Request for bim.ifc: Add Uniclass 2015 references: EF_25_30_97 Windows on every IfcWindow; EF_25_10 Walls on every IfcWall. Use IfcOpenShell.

First a look at what the model holds.

```python
import ifcopenshell

model = ifcopenshell.open("bim.ifc")
print(model.schema)
print("classifications:", [c.Name for c in model.by_type("IfcClassification")])
for ifc_class in ("IfcDoor", "IfcRoof", "IfcStair", "IfcWall", "IfcWindow"):
    print(ifc_class, len(model.by_type(ifc_class)))
```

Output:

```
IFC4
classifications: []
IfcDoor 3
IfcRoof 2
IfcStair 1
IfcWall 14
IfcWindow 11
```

```python
import ifcopenshell
import ifcopenshell.api.classification

model = ifcopenshell.open("bim.ifc")

system = ifcopenshell.api.classification.add_classification(model, classification="Uniclass 2015")

codes = {
    "IfcWindow": ("EF_25_30_97", "Windows"),
    "IfcWall": ("EF_25_10", "Walls"),
}
for ifc_class, (code, name) in codes.items():
    products = model.by_type(ifc_class)
    ifcopenshell.api.classification.add_reference(
        model, products=products, classification=system, identification=code, name=name
    )
    print(code, len(products))

model.write("bim_edited.ifc")
```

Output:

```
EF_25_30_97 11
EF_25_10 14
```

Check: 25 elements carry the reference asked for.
